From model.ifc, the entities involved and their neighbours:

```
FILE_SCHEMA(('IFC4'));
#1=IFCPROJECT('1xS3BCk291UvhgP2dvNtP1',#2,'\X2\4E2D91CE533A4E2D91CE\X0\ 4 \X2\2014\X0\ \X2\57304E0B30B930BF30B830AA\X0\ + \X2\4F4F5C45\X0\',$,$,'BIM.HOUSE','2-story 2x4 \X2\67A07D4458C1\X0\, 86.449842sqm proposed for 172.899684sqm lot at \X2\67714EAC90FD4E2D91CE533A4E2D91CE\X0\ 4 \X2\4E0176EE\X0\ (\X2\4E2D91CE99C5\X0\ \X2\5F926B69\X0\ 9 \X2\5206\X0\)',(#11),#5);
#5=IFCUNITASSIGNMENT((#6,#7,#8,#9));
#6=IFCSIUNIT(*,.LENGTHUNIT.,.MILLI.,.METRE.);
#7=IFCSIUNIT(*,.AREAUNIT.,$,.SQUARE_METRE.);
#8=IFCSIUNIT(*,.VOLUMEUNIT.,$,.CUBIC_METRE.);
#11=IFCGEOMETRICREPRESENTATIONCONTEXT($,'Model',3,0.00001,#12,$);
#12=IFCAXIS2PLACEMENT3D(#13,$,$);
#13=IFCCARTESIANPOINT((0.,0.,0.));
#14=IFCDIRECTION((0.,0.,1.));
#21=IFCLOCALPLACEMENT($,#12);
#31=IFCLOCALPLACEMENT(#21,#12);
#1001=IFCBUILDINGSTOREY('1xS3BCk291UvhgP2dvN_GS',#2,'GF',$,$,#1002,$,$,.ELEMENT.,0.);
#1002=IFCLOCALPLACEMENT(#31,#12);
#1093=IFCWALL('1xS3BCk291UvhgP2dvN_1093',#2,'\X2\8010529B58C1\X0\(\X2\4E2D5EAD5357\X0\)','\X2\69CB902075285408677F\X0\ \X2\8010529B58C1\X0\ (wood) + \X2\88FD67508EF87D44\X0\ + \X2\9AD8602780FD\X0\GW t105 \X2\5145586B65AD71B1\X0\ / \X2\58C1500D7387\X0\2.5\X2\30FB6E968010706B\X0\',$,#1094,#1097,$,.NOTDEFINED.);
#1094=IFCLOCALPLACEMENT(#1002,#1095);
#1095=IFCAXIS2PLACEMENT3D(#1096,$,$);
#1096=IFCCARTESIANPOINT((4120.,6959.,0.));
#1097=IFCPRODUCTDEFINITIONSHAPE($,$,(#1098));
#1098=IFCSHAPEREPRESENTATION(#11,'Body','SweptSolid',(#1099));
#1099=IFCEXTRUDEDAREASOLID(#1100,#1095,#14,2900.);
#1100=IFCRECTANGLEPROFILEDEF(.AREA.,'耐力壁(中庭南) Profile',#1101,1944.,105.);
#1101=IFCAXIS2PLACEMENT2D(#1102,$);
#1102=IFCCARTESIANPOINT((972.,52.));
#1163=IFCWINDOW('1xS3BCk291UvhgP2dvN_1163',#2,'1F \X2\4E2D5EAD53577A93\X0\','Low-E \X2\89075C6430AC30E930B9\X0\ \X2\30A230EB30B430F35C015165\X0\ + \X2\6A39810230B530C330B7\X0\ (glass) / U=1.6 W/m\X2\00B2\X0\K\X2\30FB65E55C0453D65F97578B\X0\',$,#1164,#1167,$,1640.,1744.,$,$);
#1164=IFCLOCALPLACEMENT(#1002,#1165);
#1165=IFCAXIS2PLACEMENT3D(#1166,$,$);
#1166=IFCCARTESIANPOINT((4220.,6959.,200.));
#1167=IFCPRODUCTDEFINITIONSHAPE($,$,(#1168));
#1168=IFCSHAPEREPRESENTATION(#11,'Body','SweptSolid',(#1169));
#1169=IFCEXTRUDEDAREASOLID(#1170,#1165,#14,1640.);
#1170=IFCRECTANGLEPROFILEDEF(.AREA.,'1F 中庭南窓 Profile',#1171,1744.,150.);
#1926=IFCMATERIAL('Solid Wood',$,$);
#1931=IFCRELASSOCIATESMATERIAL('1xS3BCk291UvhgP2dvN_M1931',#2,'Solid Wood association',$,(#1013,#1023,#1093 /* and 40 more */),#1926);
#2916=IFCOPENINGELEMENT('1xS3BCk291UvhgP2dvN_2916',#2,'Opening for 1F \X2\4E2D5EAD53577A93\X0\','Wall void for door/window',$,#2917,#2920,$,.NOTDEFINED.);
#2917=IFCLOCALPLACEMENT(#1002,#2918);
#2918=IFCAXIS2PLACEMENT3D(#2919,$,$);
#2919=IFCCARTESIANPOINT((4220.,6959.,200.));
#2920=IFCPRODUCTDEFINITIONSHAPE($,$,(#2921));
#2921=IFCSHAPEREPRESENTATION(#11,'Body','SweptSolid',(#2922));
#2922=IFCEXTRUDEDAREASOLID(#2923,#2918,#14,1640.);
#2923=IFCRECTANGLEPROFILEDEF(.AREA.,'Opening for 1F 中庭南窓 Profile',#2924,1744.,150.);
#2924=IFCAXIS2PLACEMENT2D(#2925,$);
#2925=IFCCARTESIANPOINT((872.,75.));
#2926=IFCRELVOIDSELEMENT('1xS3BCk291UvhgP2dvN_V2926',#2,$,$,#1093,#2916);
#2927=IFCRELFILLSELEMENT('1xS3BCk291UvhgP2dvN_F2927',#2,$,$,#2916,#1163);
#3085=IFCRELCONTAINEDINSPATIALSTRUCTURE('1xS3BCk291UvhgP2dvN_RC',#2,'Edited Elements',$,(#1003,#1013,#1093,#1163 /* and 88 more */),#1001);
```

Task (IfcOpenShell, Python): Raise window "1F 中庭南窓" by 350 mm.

```python
import numpy as np
import ifcopenshell
import ifcopenshell.api.geometry
import ifcopenshell.util.placement
import ifcopenshell.util.unit

model = ifcopenshell.open("model.ifc")
unit_scale = ifcopenshell.util.unit.calculate_unit_scale(model)

window = model.by_id(1163)
opening = window.FillsVoids[0].RelatingOpeningElement
dz = 0.35 / unit_scale

shift = np.array([0.0, 0.0, dz])
# The window is not placed relative to its opening, so move both.
for product in (opening, window):
    matrix = ifcopenshell.util.placement.get_local_placement(product.ObjectPlacement)
    matrix[:3, 3] += shift
    ifcopenshell.api.geometry.edit_object_placement(model, product=product, matrix=matrix, is_si=False)

print(f"moved by {dz * unit_scale:+.3f} m")

model.write("model_edited.ifc")
```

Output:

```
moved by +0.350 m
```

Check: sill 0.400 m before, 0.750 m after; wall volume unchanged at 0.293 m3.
